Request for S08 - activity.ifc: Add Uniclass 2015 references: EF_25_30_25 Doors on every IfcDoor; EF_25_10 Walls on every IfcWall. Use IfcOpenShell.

First a look at what the model holds.

```python
import ifcopenshell

model = ifcopenshell.open("S08 - activity.ifc")
print(model.schema)
print("classifications:", [c.Name for c in model.by_type("IfcClassification")])
for ifc_class in ("IfcDoor", "IfcRoof", "IfcStair", "IfcWall", "IfcWindow"):
    print(ifc_class, len(model.by_type(ifc_class)))
```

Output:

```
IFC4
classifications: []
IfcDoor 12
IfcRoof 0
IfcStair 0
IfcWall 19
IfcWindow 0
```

```python
import ifcopenshell
import ifcopenshell.api.classification

model = ifcopenshell.open("S08 - activity.ifc")

system = ifcopenshell.api.classification.add_classification(model, classification="Uniclass 2015")

codes = {
    "IfcDoor": ("EF_25_30_25", "Doors"),
    "IfcWall": ("EF_25_10", "Walls"),
}
for ifc_class, (code, name) in codes.items():
    products = model.by_type(ifc_class)
    ifcopenshell.api.classification.add_reference(
        model, products=products, classification=system, identification=code, name=name
    )
    print(code, len(products))

model.write("S08 - activity_updated.ifc")
```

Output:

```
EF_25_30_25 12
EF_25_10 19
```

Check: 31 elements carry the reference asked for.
